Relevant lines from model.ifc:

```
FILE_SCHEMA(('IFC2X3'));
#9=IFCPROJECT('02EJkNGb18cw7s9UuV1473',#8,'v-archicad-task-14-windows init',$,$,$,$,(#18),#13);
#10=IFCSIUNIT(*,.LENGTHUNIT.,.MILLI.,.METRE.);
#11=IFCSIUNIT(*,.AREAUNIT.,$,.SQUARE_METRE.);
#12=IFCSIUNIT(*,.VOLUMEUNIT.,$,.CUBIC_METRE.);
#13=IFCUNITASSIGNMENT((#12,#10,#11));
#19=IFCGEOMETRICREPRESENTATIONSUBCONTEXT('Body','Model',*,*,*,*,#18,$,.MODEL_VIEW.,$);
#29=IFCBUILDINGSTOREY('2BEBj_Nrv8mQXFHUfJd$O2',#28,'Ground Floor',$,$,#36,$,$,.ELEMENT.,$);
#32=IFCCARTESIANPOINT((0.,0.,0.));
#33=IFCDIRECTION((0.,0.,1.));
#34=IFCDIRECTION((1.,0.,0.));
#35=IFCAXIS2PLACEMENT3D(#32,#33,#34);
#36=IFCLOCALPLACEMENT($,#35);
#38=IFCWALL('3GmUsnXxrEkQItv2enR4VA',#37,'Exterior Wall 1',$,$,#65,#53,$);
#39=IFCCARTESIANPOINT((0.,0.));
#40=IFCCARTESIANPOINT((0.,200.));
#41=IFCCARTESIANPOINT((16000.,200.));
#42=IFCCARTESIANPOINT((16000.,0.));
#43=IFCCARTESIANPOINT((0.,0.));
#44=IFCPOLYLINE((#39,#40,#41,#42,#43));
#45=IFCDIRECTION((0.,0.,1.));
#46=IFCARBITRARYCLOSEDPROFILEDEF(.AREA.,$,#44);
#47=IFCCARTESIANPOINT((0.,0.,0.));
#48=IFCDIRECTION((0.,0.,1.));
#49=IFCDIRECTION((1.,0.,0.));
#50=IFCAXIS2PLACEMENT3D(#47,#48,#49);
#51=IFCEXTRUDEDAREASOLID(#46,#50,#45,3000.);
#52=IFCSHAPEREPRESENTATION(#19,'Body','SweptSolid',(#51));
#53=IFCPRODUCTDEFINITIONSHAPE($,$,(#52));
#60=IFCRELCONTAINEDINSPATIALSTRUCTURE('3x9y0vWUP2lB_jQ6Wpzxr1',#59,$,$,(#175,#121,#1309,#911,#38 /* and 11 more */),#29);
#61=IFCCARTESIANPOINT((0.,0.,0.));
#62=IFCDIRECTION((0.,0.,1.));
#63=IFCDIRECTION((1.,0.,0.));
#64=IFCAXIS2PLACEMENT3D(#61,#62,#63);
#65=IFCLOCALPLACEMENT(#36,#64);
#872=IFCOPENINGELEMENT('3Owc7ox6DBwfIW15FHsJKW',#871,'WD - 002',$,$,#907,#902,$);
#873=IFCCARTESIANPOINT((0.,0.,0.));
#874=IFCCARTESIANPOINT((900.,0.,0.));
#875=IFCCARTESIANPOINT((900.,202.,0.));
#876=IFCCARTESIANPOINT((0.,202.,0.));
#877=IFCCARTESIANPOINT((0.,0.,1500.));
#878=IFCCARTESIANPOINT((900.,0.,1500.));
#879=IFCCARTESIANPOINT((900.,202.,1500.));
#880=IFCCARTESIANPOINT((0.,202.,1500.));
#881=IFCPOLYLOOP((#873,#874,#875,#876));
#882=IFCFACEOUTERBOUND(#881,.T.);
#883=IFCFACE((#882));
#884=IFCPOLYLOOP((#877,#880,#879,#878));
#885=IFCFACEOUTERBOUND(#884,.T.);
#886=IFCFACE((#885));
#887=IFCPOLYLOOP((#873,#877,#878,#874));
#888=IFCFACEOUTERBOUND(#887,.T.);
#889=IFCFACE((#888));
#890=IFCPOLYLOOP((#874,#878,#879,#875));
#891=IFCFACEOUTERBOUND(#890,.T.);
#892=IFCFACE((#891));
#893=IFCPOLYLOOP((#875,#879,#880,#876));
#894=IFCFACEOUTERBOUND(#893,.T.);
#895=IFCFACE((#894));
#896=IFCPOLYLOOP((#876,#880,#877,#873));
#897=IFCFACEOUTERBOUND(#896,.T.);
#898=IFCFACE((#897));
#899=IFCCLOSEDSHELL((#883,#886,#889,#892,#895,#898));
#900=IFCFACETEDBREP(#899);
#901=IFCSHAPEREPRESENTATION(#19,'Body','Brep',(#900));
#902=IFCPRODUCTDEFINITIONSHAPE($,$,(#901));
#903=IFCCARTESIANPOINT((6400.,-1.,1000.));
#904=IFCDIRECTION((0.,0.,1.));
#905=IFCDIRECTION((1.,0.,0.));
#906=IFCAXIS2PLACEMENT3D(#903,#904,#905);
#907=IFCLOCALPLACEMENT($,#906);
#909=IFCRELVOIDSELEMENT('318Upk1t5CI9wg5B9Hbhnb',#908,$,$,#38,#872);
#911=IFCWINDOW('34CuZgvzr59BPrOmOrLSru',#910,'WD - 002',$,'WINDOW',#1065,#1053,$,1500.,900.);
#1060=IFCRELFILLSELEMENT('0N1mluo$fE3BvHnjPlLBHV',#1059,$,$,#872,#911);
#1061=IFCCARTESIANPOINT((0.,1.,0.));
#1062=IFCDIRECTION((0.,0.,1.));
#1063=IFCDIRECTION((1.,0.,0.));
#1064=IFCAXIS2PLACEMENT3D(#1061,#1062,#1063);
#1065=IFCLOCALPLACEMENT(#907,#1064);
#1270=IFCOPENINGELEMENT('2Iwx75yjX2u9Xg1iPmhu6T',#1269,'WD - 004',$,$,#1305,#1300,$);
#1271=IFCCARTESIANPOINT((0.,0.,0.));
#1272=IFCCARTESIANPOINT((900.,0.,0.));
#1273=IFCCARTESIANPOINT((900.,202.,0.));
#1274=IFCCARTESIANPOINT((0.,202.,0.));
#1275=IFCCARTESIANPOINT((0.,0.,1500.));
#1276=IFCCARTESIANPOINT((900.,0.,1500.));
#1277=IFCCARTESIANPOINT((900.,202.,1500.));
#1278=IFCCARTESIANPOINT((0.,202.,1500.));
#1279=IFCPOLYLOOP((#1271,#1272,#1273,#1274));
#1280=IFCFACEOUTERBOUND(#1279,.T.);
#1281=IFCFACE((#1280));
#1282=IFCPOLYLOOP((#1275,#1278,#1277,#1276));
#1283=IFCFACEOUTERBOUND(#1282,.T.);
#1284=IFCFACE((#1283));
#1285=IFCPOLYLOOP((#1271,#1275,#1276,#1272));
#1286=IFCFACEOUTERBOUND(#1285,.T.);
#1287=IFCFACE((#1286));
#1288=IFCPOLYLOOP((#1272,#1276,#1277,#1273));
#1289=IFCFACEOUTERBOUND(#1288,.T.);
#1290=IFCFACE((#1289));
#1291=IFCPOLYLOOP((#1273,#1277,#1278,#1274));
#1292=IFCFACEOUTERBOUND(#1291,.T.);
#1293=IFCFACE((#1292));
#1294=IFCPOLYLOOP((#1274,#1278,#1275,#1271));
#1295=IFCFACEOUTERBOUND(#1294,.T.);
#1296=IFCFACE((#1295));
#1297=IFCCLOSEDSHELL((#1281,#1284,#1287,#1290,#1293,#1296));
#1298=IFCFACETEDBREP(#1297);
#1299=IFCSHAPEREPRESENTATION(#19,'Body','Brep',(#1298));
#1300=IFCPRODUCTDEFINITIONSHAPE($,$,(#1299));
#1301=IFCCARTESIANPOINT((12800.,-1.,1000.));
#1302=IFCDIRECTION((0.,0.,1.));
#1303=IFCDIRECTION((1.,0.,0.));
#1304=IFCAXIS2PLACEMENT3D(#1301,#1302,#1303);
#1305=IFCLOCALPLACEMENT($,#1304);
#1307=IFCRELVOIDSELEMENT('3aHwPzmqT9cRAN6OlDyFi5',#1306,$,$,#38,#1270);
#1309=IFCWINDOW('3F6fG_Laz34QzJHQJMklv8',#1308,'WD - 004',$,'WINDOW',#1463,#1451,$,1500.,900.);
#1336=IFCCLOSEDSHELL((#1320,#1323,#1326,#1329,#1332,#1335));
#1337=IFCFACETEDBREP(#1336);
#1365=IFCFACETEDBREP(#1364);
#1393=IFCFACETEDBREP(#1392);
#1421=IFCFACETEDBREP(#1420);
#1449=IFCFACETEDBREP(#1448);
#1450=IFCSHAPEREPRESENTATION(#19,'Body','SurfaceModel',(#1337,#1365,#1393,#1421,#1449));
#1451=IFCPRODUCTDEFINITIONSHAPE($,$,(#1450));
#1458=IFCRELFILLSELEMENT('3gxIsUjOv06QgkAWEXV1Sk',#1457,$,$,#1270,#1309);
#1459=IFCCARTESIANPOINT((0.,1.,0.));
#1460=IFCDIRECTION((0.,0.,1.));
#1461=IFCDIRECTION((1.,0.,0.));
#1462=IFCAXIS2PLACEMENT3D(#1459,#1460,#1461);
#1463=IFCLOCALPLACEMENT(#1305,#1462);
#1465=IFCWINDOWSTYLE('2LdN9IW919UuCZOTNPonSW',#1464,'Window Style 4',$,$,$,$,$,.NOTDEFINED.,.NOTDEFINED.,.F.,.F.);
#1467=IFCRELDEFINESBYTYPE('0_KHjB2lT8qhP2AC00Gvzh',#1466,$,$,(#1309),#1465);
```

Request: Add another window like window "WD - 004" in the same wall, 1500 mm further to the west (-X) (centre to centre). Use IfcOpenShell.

```python
import ifcopenshell
import ifcopenshell.api.feature
import ifcopenshell.api.geometry
import ifcopenshell.api.root
import ifcopenshell.geom
import ifcopenshell.util.element
import ifcopenshell.util.placement
import ifcopenshell.util.shape

model = ifcopenshell.open("model.ifc")
settings = ifcopenshell.geom.settings()


def volume(element):
    """Net volume in cubic metres, openings subtracted."""
    shape = ifcopenshell.geom.create_shape(settings, element)
    return ifcopenshell.util.shape.get_volume(shape.geometry)


window = model.by_guid("3F6fG_Laz34QzJHQJMklv8")
opening = window.FillsVoids[0].RelatingOpeningElement
wall = opening.VoidsElements[0].RelatingBuildingElement
before = volume(wall)
shift = ifcopenshell.util.placement.get_local_placement(wall.ObjectPlacement)[:3, 0] * -1500.0

# copy_class copies the void relationship, type, container and properties, but no geometry.
new_opening = ifcopenshell.api.root.copy_class(model, product=opening)
new_opening.Representation = ifcopenshell.util.element.copy_deep(
    model, opening.Representation, exclude=["IfcGeometricRepresentationContext", "IfcRepresentationMap"]
)
new_window = ifcopenshell.api.root.copy_class(model, product=window)
new_window.Representation = ifcopenshell.util.element.copy_deep(
    model, window.Representation, exclude=["IfcGeometricRepresentationContext", "IfcRepresentationMap"]
)
fills = ifcopenshell.api.feature.add_filling(model, opening=new_opening, element=new_window)
fills.OwnerHistory = new_window.OwnerHistory  # required in IFC2X3

for old, new in ((opening, new_opening), (window, new_window)):
    matrix = ifcopenshell.util.placement.get_local_placement(old.ObjectPlacement)
    matrix[:3, 3] += shift
    ifcopenshell.api.geometry.edit_object_placement(model, product=new, matrix=matrix, is_si=False)

after = volume(wall)

print(f"wall volume {before:.3f} -> {after:.3f} m3")

model.write("model_updated.ifc")
```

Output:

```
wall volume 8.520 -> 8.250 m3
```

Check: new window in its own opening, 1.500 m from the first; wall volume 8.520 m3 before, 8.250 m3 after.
